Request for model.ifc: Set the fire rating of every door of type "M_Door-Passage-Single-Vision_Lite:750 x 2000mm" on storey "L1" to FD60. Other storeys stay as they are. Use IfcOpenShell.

First a look at what the model holds.

```python
import ifcopenshell
import ifcopenshell.util.element

model = ifcopenshell.open("model.ifc")
print(model.schema)
storey = next(s for s in model.by_type("IfcBuildingStorey") if s.Name == "L1")
doors = [e for e in ifcopenshell.util.element.get_decomposition(storey) if e.is_a("IfcDoor")]
seen = {}
for e in doors:
    element_type = ifcopenshell.util.element.get_type(e)
    key = (element_type.Name if element_type != e and element_type else None, ifcopenshell.util.element.get_pset(e, "Pset_DoorCommon", "FireRating"))
    seen[key] = seen.get(key, 0) + 1
for (name, value), count in sorted(seen.items(), key=str):
    print(count, "x", name, "|", value)
```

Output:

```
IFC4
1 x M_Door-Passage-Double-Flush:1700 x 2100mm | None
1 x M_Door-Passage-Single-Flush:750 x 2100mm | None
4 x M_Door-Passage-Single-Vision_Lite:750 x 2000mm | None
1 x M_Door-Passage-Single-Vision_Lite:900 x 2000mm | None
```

```python
import ifcopenshell
import ifcopenshell.api.pset
import ifcopenshell.util.element

model = ifcopenshell.open("model.ifc")

storey = next(s for s in model.by_type("IfcBuildingStorey") if s.Name == "L1")
doors = [e for e in ifcopenshell.util.element.get_decomposition(storey) if e.is_a("IfcDoor")]

count = 0
for e in doors:
    element_type = ifcopenshell.util.element.get_type(e)
    if element_type in (None, e) or element_type.Name != "M_Door-Passage-Single-Vision_Lite:750 x 2000mm":
        continue
    # add_pset returns the element's existing set when there is one.
    pset = ifcopenshell.api.pset.add_pset(model, product=e, name="Pset_DoorCommon")
    ifcopenshell.api.pset.edit_pset(model, pset=pset, properties={"FireRating": "FD60"})
    count += 1

print(count, "doors updated")

model.write("model-out.ifc")
```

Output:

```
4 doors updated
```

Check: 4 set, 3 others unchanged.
